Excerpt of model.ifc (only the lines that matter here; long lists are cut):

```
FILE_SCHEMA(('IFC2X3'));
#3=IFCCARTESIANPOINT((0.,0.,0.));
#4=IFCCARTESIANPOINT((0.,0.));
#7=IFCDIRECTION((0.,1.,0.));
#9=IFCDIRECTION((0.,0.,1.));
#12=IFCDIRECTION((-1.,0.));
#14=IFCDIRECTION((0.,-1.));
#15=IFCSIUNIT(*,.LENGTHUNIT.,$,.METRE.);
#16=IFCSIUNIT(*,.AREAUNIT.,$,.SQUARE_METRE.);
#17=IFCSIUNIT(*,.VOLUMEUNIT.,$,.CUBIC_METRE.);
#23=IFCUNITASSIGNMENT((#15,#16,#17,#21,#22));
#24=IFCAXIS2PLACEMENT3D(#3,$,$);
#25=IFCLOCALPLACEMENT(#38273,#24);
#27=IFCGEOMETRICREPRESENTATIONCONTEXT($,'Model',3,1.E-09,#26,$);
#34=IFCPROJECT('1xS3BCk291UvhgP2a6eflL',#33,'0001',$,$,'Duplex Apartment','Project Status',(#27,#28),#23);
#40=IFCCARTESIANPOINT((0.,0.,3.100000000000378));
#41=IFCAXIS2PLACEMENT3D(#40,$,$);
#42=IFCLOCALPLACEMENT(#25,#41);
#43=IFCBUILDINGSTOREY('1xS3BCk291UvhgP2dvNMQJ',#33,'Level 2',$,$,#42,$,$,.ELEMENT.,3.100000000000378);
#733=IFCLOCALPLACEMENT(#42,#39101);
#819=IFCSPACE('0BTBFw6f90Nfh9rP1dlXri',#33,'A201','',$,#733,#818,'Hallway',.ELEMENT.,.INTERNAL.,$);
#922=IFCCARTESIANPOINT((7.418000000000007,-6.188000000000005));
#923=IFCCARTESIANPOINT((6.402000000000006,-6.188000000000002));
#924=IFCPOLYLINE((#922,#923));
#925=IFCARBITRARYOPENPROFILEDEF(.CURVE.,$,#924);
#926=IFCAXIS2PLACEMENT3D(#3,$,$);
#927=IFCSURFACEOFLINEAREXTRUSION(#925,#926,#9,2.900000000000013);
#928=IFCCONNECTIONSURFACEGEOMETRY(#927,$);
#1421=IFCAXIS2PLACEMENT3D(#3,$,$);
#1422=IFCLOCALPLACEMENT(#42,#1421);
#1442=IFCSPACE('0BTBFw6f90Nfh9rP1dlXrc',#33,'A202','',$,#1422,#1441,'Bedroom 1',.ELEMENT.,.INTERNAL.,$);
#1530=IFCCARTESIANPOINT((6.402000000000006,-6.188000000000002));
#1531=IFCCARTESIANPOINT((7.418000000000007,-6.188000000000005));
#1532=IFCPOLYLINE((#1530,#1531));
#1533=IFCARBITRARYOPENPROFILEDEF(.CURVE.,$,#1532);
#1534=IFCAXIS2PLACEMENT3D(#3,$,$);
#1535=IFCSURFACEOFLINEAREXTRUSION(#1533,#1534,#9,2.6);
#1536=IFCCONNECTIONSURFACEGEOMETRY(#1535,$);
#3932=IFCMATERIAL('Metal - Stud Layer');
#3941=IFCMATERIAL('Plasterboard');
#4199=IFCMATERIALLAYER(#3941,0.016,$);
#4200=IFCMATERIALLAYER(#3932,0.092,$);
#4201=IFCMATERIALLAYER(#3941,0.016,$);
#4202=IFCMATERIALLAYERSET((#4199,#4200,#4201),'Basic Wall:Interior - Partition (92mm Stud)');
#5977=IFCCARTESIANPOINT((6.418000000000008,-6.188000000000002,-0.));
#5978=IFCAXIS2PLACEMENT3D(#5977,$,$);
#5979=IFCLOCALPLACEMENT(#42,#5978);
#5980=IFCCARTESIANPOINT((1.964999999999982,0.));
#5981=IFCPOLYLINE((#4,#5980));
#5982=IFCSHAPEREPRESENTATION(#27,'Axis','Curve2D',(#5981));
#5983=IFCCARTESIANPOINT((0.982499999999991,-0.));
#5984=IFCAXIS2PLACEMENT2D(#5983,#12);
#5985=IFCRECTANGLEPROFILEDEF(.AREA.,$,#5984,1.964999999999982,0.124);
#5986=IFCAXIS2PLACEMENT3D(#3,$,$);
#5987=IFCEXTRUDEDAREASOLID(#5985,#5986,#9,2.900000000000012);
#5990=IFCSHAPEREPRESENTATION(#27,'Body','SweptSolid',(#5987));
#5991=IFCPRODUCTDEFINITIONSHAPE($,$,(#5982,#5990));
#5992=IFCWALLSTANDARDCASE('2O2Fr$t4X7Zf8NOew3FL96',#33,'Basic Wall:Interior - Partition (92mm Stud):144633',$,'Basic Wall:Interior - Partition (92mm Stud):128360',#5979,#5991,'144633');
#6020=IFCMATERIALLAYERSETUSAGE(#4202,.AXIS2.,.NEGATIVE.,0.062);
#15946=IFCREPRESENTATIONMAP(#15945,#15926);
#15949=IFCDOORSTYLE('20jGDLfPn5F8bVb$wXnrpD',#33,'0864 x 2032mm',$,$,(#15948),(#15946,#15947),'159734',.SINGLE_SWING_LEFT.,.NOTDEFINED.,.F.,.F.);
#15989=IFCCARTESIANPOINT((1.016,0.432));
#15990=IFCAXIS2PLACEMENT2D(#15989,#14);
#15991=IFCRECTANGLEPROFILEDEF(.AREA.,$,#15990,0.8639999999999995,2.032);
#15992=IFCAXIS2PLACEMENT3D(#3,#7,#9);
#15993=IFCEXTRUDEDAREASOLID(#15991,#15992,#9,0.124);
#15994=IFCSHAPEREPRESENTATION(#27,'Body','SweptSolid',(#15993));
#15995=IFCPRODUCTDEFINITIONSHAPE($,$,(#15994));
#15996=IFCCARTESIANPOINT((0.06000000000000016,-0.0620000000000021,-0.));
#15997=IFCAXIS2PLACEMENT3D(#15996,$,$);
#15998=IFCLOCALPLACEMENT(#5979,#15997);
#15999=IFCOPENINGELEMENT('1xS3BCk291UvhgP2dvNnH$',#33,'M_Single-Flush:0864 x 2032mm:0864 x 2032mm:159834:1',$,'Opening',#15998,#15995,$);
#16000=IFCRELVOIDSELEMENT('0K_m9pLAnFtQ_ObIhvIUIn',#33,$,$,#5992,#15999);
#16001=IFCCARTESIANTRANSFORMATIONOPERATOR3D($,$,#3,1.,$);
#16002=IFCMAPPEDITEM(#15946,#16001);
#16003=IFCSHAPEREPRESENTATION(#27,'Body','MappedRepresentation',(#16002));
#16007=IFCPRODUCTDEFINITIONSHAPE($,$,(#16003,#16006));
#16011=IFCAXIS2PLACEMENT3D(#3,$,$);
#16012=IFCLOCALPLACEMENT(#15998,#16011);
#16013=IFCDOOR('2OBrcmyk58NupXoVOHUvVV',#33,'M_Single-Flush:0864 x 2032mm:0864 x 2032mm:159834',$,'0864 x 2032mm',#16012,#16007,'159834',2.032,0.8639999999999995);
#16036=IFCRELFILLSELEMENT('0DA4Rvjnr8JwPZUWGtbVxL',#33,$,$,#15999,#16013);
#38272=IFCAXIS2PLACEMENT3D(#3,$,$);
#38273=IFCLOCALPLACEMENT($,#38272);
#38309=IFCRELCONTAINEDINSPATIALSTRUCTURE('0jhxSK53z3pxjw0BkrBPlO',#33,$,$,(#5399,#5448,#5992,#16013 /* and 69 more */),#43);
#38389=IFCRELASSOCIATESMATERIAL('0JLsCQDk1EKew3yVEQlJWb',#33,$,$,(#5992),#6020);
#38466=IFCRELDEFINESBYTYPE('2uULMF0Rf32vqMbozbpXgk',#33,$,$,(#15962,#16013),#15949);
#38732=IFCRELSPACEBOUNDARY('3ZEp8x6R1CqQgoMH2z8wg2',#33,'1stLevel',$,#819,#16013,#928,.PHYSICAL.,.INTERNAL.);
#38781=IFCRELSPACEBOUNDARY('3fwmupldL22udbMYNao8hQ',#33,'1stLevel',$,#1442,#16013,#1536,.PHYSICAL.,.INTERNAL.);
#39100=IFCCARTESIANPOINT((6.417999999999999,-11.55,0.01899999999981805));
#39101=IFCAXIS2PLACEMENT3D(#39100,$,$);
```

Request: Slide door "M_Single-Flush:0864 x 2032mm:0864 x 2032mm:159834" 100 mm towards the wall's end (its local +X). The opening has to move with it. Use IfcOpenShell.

```python
import numpy as np
import ifcopenshell
import ifcopenshell.api.geometry
import ifcopenshell.util.placement

model = ifcopenshell.open("model.ifc")

door = model.by_guid("2OBrcmyk58NupXoVOHUvVV")
opening = door.FillsVoids[0].RelatingOpeningElement
wall = opening.VoidsElements[0].RelatingBuildingElement

wall_matrix = ifcopenshell.util.placement.get_local_placement(wall.ObjectPlacement)
shift = wall_matrix[:3, 0] * 0.1
before = ifcopenshell.util.placement.get_local_placement(door.ObjectPlacement)[:3, 3].copy()

# The door is placed relative to its opening, so it follows when the opening moves.
matrix = ifcopenshell.util.placement.get_local_placement(opening.ObjectPlacement)
matrix[:3, 3] += shift
ifcopenshell.api.geometry.edit_object_placement(
    model, product=opening, matrix=matrix, is_si=False, should_transform_children=True
)

# Space boundary surfaces are stored in each space's coordinates; move them too.
for rel in door.ProvidesBoundaries:
    if not rel.ConnectionGeometry:
        continue
    surface = rel.ConnectionGeometry.SurfaceOnRelatingElement
    space_matrix = ifcopenshell.util.placement.get_local_placement(rel.RelatingSpace.ObjectPlacement)
    point = np.array(surface.Position.Location.Coordinates) + space_matrix[:3, :3].T @ shift
    surface.Position = model.createIfcAxis2Placement3D(
        model.createIfcCartesianPoint(point.tolist()), surface.Position.Axis, surface.Position.RefDirection
    )

after = ifcopenshell.util.placement.get_local_placement(door.ObjectPlacement)[:3, 3]
print("door moved by", (after - before).round(3) + 0.0)

model.write("model-out.ifc")
```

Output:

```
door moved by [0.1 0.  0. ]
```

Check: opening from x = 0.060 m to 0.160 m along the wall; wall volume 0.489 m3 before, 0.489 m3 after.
